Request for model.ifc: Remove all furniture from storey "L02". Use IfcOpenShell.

First a look at what the model holds.

```python
import ifcopenshell
import ifcopenshell.util.element

model = ifcopenshell.open("model.ifc")
print(model.schema)
storey = next(s for s in model.by_type("IfcBuildingStorey") if s.Name == "L02")
furniture = [e for e in ifcopenshell.util.element.get_decomposition(storey) if e.is_a("IfcFurnishingElement")]
seen = {}
for e in furniture:
    element_type = ifcopenshell.util.element.get_type(e)
    name = element_type.Name if element_type not in (None, e) else None
    seen[name] = seen.get(name, 0) + 1
for name, count in sorted(seen.items(), key=str):
    print(count, "x", name)
```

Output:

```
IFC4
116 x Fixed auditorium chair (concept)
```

```python
import ifcopenshell
import ifcopenshell.api.root
import ifcopenshell.util.element

model = ifcopenshell.open("model.ifc")

storey = next(s for s in model.by_type("IfcBuildingStorey") if s.Name == "L02")
furniture = [e for e in ifcopenshell.util.element.get_decomposition(storey) if e.is_a("IfcFurnishingElement")]

for e in furniture:
    ifcopenshell.api.root.remove_product(model, product=e)
print(len(furniture), "removed")

model.write("model-out.ifc")
```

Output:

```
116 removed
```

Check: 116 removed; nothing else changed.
